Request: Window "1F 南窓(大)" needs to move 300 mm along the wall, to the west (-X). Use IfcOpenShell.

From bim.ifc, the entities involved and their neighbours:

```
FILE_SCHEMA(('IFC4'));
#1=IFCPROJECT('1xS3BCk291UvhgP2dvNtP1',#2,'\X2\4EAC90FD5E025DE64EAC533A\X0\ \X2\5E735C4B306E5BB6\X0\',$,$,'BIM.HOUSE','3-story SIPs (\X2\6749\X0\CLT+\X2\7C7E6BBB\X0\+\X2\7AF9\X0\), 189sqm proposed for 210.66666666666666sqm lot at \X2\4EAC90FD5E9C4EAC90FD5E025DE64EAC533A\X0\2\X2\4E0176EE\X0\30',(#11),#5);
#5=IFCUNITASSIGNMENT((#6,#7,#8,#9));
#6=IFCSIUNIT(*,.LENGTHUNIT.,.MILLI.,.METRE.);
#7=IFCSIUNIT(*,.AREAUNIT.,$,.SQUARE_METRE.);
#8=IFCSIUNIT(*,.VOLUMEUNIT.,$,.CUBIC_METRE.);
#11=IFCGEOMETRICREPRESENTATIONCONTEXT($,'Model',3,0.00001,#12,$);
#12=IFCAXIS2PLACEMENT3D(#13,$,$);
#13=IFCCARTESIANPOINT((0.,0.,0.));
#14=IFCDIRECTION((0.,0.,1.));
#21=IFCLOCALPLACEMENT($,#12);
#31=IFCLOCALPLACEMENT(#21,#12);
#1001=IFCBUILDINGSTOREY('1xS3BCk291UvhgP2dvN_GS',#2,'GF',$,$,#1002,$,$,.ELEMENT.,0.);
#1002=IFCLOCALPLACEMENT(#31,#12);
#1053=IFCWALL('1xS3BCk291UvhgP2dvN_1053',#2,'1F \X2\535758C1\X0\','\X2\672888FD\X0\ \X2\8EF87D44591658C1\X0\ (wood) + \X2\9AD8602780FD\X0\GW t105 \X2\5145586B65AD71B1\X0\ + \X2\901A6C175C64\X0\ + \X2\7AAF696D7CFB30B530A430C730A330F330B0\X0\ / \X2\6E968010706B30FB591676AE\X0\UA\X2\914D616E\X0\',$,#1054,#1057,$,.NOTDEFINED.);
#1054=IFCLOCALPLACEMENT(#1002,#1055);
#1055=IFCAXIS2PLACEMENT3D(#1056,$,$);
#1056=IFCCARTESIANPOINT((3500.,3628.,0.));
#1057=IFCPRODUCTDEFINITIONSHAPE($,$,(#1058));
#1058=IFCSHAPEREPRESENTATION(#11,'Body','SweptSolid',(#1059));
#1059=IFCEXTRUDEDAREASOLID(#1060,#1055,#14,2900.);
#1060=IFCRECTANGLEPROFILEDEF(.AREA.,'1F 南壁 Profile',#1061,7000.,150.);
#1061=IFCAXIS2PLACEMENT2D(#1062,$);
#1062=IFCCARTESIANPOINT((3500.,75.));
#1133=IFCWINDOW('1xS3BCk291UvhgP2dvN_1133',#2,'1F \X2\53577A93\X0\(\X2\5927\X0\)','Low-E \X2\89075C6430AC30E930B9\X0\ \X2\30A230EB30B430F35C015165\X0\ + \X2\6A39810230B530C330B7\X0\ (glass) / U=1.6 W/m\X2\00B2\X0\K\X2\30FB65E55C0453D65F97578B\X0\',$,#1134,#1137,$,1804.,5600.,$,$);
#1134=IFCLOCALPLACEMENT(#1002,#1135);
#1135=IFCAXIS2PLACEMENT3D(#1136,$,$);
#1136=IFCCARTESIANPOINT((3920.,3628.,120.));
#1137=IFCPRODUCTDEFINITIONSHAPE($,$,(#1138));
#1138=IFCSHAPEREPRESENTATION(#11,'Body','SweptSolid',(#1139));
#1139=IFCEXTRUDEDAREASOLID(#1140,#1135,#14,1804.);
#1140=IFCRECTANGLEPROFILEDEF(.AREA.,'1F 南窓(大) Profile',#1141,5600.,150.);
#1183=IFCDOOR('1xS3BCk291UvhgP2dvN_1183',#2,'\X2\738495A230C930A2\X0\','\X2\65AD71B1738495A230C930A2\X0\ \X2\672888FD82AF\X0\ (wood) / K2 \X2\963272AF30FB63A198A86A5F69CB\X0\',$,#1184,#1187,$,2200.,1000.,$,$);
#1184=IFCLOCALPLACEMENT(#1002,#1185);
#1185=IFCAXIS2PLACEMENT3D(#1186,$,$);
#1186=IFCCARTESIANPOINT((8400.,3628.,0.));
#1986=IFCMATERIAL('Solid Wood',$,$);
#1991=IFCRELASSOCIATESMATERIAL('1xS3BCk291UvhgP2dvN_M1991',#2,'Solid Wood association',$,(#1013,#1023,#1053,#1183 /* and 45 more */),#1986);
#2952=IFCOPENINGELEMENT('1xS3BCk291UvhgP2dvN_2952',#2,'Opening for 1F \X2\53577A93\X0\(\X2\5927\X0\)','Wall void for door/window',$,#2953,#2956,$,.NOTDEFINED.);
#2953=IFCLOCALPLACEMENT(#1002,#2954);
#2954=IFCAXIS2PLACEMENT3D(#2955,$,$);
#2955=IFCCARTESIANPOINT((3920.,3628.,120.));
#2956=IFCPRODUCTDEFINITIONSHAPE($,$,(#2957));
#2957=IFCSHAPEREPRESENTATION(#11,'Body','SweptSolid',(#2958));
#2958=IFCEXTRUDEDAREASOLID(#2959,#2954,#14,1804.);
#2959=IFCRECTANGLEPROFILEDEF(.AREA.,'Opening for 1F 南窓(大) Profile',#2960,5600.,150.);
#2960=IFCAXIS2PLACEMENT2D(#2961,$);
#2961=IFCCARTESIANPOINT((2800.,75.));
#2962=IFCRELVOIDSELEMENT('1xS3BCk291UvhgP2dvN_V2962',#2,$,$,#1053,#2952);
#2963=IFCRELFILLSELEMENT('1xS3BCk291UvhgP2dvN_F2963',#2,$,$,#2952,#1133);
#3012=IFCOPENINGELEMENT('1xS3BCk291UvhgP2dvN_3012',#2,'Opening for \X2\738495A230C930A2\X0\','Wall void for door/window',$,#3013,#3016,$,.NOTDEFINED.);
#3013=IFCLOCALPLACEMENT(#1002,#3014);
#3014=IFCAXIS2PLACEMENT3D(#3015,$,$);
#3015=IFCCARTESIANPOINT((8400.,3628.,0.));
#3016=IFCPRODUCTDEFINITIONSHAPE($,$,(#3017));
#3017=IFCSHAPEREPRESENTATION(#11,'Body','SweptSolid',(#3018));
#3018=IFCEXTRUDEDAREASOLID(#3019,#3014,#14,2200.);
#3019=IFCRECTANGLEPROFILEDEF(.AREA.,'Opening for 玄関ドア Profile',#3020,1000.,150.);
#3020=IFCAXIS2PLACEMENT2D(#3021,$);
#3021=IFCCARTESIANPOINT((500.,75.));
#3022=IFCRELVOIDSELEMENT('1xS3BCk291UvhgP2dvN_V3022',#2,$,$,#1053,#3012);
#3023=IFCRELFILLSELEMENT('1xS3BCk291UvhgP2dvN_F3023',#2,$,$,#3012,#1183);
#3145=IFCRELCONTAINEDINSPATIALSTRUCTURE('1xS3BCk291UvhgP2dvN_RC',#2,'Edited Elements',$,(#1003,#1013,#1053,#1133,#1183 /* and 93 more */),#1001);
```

```python
import ifcopenshell
import ifcopenshell.api.geometry
import ifcopenshell.util.placement
import ifcopenshell.util.unit

model = ifcopenshell.open("bim.ifc")
unit_scale = ifcopenshell.util.unit.calculate_unit_scale(model)

window = model.by_guid("1xS3BCk291UvhgP2dvN_1133")
opening = window.FillsVoids[0].RelatingOpeningElement
wall = opening.VoidsElements[0].RelatingBuildingElement

wall_matrix = ifcopenshell.util.placement.get_local_placement(wall.ObjectPlacement)
shift = wall_matrix[:3, 0] * -0.3 / unit_scale
before = ifcopenshell.util.placement.get_local_placement(window.ObjectPlacement)[:3, 3].copy()

# The window is not placed relative to its opening, so move both.
for product in (opening, window):
    matrix = ifcopenshell.util.placement.get_local_placement(product.ObjectPlacement)
    matrix[:3, 3] += shift
    ifcopenshell.api.geometry.edit_object_placement(model, product=product, matrix=matrix, is_si=False)

after = ifcopenshell.util.placement.get_local_placement(window.ObjectPlacement)[:3, 3]
print("window moved by", (after - before).round(3) + 0.0)

model.write("bim_edited.ifc")
```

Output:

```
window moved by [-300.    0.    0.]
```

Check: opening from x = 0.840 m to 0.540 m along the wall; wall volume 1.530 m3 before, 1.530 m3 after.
